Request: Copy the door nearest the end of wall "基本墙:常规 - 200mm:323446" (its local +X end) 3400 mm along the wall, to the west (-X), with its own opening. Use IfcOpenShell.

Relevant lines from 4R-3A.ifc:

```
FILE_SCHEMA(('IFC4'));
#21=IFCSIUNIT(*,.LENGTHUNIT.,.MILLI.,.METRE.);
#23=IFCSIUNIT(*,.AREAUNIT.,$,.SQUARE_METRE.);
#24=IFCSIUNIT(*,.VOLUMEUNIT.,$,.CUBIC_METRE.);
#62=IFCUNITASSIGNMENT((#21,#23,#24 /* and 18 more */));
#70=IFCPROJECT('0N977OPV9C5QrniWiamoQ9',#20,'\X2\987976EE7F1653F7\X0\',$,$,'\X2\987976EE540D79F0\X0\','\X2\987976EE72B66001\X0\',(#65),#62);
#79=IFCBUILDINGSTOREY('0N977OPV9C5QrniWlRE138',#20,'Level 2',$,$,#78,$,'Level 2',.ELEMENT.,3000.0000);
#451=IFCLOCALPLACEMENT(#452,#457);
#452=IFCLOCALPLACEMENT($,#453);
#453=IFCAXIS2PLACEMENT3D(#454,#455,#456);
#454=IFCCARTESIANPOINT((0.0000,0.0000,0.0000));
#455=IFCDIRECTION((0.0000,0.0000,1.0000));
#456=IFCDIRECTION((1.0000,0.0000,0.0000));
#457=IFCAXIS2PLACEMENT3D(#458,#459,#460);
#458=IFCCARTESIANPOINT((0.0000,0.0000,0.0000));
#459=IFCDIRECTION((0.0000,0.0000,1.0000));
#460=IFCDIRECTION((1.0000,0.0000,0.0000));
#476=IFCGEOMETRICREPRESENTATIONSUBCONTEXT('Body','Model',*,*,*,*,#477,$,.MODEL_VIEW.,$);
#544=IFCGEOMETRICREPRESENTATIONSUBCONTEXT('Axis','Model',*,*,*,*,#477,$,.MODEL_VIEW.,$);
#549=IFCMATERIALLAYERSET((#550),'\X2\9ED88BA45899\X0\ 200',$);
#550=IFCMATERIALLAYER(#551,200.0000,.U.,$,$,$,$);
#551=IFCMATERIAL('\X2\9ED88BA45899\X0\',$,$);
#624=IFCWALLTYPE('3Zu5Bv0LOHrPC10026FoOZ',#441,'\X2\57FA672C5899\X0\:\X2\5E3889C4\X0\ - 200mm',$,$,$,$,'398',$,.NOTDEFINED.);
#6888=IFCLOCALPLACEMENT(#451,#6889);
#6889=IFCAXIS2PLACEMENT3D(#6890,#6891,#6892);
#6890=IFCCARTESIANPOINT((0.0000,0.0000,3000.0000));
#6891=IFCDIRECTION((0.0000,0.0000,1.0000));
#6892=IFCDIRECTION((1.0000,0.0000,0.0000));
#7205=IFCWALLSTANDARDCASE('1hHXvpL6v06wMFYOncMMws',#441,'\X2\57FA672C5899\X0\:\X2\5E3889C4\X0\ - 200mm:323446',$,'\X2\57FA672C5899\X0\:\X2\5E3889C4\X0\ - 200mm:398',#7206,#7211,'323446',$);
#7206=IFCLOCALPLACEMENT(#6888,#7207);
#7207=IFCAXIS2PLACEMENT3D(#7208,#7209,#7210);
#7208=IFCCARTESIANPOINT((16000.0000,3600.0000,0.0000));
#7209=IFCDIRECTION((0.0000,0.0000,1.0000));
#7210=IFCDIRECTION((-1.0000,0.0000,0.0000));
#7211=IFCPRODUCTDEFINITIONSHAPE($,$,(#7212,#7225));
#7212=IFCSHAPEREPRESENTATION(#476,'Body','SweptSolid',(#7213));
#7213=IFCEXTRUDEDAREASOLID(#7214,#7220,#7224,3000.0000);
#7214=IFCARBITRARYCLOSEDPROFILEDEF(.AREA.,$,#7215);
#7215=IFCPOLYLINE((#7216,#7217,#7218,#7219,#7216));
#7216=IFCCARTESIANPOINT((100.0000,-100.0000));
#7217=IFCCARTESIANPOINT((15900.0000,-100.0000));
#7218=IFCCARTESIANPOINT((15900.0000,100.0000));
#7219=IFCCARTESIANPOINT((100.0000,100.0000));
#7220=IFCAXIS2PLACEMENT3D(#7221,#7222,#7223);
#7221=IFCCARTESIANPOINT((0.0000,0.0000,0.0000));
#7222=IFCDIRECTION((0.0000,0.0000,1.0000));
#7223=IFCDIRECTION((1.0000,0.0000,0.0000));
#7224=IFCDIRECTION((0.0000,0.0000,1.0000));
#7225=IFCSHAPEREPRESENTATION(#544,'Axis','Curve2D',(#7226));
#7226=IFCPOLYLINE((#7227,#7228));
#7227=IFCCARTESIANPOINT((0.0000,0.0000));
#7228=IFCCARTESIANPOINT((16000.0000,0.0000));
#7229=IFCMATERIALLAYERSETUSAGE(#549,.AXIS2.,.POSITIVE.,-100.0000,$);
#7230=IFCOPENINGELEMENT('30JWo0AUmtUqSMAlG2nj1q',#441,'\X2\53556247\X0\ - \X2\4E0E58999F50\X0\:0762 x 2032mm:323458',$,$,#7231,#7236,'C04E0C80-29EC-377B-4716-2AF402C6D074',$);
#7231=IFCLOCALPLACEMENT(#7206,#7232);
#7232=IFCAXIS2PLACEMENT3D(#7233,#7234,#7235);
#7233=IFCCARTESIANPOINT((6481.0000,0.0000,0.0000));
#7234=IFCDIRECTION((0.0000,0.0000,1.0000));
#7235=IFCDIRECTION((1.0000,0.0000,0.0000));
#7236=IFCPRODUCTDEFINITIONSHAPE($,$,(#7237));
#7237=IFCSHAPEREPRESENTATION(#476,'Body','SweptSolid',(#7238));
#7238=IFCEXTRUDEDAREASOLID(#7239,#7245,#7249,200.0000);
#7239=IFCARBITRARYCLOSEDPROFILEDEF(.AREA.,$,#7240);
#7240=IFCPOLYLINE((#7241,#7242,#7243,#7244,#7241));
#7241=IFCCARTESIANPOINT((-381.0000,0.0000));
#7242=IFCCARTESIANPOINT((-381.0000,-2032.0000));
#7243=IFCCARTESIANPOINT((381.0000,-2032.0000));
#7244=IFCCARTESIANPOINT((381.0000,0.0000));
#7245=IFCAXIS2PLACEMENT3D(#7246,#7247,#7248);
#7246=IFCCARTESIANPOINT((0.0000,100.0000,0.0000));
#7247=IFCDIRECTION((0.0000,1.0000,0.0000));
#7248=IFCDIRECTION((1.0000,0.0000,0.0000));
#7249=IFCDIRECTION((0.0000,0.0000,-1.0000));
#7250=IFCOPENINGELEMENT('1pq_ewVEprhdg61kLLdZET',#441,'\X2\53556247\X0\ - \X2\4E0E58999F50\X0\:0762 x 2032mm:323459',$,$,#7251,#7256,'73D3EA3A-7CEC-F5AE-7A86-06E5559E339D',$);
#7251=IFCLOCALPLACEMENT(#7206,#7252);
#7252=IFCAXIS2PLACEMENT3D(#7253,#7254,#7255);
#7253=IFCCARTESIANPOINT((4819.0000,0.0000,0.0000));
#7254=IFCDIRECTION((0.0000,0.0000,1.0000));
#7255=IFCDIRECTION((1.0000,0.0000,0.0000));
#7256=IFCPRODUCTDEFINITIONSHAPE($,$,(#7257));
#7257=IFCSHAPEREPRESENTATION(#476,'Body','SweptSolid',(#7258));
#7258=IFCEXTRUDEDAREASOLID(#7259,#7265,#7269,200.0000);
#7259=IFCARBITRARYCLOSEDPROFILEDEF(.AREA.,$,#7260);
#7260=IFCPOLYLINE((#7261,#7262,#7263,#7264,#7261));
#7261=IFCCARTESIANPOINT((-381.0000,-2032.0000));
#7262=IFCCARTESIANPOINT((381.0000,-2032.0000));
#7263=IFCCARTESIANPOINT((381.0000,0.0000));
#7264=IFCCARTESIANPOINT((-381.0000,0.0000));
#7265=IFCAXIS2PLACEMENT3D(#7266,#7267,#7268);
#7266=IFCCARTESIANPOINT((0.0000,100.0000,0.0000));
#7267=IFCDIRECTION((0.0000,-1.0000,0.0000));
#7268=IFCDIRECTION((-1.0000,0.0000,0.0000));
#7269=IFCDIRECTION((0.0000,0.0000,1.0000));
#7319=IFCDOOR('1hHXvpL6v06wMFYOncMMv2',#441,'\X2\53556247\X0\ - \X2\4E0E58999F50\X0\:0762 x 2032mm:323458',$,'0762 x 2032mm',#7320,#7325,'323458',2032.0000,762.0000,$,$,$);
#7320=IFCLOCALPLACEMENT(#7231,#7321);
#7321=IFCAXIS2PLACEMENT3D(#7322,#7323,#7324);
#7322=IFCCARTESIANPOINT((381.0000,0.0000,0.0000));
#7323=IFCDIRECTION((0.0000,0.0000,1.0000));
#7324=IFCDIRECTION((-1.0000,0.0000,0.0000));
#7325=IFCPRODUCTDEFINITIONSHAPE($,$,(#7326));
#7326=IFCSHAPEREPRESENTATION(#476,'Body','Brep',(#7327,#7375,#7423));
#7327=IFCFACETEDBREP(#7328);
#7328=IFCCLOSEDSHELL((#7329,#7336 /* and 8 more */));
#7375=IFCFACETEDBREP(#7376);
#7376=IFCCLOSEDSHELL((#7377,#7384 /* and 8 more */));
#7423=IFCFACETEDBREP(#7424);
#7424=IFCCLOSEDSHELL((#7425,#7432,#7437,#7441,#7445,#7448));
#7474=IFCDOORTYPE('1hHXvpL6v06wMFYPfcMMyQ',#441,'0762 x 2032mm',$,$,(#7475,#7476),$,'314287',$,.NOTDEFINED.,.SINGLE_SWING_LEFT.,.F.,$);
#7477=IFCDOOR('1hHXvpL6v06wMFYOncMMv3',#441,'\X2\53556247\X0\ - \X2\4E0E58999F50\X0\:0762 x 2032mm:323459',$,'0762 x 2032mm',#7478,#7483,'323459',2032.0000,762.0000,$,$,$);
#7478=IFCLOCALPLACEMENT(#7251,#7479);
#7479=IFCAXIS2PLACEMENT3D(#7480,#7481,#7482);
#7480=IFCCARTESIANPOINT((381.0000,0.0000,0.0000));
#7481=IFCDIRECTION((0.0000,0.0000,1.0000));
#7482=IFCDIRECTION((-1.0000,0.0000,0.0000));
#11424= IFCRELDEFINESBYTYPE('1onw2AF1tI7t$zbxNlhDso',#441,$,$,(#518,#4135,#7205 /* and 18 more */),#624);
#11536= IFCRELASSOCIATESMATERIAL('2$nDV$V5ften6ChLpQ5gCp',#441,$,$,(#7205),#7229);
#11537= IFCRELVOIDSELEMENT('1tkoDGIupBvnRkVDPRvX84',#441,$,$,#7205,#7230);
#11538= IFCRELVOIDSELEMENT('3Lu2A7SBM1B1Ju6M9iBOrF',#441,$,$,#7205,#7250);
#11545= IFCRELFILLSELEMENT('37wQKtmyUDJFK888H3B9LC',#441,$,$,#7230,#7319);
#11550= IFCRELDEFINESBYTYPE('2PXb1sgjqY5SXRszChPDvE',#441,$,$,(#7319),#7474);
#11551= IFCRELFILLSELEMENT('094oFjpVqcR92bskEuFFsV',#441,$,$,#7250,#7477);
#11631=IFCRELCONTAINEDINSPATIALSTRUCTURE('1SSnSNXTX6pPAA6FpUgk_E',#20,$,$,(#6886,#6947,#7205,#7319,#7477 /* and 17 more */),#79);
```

```python
import ifcopenshell
import ifcopenshell.api.feature
import ifcopenshell.api.geometry
import ifcopenshell.api.root
import ifcopenshell.geom
import ifcopenshell.util.element
import ifcopenshell.util.placement
import ifcopenshell.util.shape

model = ifcopenshell.open("4R-3A.ifc")
settings = ifcopenshell.geom.settings()


def volume(element):
    """Net volume in cubic metres, openings subtracted."""
    shape = ifcopenshell.geom.create_shape(settings, element)
    return ifcopenshell.util.shape.get_volume(shape.geometry)


def reuse_history(source, copy):
    """copy_class also copies each property set's owner history, people and application; keep the originals."""
    for rel in copy.IsDefinedBy:
        if rel.is_a("IfcRelDefinesByProperties") and (history := rel.RelatingPropertyDefinition.OwnerHistory):
            rel.RelatingPropertyDefinition.OwnerHistory = source.OwnerHistory
            ifcopenshell.util.element.remove_deep2(model, history)


door = model.by_guid("1hHXvpL6v06wMFYOncMMv2")
opening = door.FillsVoids[0].RelatingOpeningElement
wall = opening.VoidsElements[0].RelatingBuildingElement
before = volume(wall)
shift = ifcopenshell.util.placement.get_local_placement(wall.ObjectPlacement)[:3, 0] * 3400.0

# copy_class copies the void relationship, type, container and properties, but no geometry.
new_opening = ifcopenshell.api.root.copy_class(model, product=opening)
new_opening.Representation = ifcopenshell.util.element.copy_deep(
    model, opening.Representation, exclude=["IfcGeometricRepresentationContext", "IfcRepresentationMap"]
)
new_opening.Name = "单扇 - 与墙齐:0762 x 2032mm"
new_opening.Tag = None
new_door = ifcopenshell.api.root.copy_class(model, product=door)
new_door.Representation = ifcopenshell.util.element.copy_deep(
    model, door.Representation, exclude=["IfcGeometricRepresentationContext", "IfcRepresentationMap"]
)
new_door.Name = "单扇 - 与墙齐:0762 x 2032mm"
new_door.Tag = None
reuse_history(door, new_door)
ifcopenshell.api.feature.add_filling(model, opening=new_opening, element=new_door)

for old, new in ((opening, new_opening), (door, new_door)):
    matrix = ifcopenshell.util.placement.get_local_placement(old.ObjectPlacement)
    matrix[:3, 3] += shift
    ifcopenshell.api.geometry.edit_object_placement(model, product=new, matrix=matrix, is_si=False)

after = volume(wall)

print(f"wall volume {before:.3f} -> {after:.3f} m3")

model.write("4R-3A_rev.ifc")
```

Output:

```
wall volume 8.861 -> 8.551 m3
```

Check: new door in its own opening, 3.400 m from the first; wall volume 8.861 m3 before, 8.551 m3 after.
